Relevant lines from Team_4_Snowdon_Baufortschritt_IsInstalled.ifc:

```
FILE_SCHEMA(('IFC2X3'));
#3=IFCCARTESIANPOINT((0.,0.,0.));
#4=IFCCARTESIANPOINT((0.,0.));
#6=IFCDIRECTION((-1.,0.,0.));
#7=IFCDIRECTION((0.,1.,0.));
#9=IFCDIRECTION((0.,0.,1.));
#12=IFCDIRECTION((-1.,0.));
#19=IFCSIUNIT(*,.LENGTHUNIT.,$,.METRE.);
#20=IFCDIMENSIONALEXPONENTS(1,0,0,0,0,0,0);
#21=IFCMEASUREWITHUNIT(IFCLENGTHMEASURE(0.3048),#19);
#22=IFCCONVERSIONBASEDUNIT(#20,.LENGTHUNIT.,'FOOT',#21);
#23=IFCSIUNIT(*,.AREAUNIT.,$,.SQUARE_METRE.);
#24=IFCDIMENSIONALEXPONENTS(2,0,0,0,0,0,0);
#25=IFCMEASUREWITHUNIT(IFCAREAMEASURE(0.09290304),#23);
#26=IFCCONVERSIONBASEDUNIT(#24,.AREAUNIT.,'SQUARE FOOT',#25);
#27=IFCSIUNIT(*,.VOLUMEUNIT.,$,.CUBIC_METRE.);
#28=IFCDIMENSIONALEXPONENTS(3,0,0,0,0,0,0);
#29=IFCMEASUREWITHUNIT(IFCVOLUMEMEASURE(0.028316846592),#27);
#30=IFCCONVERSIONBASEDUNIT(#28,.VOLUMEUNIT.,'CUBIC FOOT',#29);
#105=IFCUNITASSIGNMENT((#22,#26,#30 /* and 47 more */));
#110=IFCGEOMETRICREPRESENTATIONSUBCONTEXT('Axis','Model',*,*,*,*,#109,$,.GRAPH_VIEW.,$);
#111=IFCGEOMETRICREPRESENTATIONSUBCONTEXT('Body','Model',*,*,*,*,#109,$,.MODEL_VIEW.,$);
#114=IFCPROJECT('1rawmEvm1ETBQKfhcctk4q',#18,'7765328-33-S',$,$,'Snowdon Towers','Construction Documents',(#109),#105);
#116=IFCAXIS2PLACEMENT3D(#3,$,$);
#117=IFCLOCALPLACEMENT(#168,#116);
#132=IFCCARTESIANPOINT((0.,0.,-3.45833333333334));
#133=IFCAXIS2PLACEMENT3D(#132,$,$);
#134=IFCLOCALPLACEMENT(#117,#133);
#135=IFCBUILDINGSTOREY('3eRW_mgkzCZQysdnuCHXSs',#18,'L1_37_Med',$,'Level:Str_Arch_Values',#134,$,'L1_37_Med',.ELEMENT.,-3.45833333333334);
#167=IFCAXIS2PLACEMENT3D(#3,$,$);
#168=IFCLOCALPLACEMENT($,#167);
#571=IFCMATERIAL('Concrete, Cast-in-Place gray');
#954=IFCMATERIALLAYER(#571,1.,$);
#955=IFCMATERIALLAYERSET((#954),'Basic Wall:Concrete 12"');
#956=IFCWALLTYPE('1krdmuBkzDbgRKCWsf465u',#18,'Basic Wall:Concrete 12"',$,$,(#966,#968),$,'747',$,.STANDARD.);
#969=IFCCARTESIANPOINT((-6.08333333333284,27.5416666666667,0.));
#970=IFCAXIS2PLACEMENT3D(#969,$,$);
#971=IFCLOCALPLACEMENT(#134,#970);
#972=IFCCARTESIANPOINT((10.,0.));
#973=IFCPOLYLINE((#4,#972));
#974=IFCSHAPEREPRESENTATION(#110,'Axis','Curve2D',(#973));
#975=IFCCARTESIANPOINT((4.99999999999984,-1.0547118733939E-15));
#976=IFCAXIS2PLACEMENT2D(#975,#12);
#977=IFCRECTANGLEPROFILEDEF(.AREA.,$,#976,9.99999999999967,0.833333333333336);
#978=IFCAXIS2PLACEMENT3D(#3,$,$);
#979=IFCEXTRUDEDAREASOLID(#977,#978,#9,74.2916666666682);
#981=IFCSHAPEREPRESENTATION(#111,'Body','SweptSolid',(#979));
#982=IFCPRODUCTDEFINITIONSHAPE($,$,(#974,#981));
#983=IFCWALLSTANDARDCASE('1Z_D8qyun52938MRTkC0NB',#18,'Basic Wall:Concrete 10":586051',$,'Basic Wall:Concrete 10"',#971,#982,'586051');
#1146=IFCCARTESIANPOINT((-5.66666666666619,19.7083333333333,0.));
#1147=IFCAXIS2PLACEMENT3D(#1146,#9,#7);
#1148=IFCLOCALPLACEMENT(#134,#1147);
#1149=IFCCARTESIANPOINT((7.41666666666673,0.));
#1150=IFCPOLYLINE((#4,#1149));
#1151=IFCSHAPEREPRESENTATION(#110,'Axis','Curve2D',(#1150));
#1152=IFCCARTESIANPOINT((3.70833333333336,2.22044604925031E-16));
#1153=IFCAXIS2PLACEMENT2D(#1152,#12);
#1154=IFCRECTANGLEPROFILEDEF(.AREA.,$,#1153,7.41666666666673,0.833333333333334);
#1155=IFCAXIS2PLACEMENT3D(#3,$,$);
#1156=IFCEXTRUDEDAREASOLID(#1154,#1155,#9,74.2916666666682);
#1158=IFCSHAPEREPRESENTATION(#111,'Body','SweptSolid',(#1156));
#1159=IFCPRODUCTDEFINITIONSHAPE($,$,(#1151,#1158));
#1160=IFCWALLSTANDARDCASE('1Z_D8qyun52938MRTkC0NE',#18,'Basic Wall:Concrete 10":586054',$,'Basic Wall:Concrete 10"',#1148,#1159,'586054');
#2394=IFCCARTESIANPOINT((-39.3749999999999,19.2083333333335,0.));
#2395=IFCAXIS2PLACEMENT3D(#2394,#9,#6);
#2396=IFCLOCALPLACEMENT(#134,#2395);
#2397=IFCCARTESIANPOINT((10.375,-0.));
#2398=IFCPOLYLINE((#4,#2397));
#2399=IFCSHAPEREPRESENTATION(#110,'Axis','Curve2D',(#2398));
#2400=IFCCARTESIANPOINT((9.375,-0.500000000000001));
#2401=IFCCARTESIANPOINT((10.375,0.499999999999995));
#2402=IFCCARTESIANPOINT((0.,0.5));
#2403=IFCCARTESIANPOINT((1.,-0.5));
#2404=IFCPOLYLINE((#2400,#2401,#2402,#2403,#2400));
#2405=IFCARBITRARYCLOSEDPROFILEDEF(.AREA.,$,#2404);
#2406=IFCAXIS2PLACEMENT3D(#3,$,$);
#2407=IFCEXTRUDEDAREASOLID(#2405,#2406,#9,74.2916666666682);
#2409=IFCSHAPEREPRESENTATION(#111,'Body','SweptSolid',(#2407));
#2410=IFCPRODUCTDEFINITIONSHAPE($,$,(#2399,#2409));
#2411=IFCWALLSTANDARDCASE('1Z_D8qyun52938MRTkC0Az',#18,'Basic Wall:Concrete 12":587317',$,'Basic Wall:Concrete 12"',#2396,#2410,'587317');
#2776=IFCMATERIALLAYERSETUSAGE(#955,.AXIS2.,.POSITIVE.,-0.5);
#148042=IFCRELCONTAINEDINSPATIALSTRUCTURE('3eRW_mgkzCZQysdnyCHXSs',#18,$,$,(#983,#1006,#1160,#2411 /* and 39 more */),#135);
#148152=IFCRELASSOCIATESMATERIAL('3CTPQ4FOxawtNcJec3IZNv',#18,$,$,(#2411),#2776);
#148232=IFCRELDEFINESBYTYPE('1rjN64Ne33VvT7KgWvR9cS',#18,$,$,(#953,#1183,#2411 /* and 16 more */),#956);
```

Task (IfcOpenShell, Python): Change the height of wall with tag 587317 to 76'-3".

```python
import ifcopenshell
import ifcopenshell.geom
import ifcopenshell.util.representation
import ifcopenshell.util.shape
import ifcopenshell.util.unit

model = ifcopenshell.open("Team_4_Snowdon_Baufortschritt_IsInstalled.ifc")
unit_scale = ifcopenshell.util.unit.calculate_unit_scale(model)
settings = ifcopenshell.geom.settings()


def volume(element):
    """Net volume in cubic metres, openings subtracted."""
    shape = ifcopenshell.geom.create_shape(settings, element)
    return ifcopenshell.util.shape.get_volume(shape.geometry)


wall = model.by_guid("1Z_D8qyun52938MRTkC0Az")
before = volume(wall)

body = ifcopenshell.util.representation.get_representation(wall, "Model", "Body")
solid = body.Items[0]
old_height = solid.Depth
solid.Depth = 915 * 0.0254 / unit_scale
after = volume(wall)

print(f"height {old_height:g} -> {solid.Depth:g}, volume {before:.3f} -> {after:.3f} m3")

model.write("Team_4_Snowdon_Baufortschritt_IsInstalled_edited.ifc")
```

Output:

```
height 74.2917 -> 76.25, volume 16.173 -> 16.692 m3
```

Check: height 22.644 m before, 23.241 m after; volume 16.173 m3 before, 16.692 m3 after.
